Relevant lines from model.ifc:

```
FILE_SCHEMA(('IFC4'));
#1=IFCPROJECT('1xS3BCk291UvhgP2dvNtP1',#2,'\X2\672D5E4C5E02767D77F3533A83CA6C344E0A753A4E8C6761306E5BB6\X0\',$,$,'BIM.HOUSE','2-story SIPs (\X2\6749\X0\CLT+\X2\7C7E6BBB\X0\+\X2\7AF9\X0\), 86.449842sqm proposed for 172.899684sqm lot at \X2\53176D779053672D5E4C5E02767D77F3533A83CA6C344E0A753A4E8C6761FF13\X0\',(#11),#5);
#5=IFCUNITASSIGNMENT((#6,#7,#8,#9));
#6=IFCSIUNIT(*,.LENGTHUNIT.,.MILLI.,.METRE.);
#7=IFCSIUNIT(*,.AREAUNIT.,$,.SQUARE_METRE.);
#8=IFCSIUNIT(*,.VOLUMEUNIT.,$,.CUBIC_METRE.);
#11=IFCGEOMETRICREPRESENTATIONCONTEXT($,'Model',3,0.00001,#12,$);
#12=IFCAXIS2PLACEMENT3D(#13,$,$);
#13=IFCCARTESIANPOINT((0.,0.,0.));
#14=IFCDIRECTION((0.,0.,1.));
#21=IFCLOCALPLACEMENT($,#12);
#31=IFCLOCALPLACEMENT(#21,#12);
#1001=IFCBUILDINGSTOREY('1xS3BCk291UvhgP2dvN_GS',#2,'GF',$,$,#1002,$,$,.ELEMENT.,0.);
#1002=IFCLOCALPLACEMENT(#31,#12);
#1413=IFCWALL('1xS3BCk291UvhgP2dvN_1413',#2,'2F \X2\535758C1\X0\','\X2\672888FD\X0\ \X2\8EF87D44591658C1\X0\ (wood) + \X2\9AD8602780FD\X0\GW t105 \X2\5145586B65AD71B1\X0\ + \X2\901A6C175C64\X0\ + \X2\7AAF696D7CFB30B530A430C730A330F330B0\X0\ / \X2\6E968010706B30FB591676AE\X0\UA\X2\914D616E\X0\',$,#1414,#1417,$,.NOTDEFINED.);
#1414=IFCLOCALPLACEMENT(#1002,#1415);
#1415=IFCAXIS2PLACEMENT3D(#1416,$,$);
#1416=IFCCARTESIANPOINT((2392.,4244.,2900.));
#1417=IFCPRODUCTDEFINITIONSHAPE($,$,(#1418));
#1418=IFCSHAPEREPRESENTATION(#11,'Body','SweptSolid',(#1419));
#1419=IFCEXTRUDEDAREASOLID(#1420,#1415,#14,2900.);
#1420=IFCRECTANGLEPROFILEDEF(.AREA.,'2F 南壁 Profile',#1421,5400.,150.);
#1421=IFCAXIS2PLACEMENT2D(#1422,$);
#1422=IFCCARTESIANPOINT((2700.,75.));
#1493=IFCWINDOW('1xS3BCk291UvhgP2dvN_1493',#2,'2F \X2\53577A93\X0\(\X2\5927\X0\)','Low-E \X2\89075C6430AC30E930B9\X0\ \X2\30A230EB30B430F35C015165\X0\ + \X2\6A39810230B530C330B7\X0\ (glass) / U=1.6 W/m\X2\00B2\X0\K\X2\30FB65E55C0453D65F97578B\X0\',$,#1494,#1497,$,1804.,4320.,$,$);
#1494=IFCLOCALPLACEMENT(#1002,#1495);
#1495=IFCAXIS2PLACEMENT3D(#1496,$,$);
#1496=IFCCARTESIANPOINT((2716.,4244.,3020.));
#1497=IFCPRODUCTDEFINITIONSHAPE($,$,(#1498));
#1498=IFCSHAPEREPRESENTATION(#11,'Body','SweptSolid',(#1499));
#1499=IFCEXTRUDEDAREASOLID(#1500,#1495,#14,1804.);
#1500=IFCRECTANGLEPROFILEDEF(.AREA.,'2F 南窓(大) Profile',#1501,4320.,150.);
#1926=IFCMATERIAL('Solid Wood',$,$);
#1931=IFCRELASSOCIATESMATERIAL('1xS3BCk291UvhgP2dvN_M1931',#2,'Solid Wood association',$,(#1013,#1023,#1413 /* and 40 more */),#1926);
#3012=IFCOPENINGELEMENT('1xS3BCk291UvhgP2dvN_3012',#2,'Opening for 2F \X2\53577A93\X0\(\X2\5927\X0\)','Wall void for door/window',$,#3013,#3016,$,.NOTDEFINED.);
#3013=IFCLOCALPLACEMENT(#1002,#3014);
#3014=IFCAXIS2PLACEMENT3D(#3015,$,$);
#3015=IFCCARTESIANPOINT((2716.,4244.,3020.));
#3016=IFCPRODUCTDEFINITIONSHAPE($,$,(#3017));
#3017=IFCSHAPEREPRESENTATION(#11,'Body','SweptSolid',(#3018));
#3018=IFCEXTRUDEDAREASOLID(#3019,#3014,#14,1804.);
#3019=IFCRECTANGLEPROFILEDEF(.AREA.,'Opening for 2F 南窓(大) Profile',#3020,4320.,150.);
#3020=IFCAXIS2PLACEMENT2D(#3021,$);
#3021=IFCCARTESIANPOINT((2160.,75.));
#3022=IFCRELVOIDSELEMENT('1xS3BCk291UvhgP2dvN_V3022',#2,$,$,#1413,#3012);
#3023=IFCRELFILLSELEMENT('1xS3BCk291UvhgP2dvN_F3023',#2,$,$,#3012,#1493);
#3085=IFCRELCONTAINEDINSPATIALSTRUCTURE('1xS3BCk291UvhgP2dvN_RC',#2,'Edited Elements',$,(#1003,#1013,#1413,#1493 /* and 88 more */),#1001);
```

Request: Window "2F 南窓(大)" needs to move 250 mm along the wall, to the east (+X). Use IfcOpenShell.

```python
import ifcopenshell
import ifcopenshell.api.geometry
import ifcopenshell.util.placement

model = ifcopenshell.open("model.ifc")

window = model.by_guid("1xS3BCk291UvhgP2dvN_1493")
opening = window.FillsVoids[0].RelatingOpeningElement
wall = opening.VoidsElements[0].RelatingBuildingElement

wall_matrix = ifcopenshell.util.placement.get_local_placement(wall.ObjectPlacement)
shift = wall_matrix[:3, 0] * 250.0
before = ifcopenshell.util.placement.get_local_placement(window.ObjectPlacement)[:3, 3].copy()

# The window is not placed relative to its opening, so move both.
for product in (opening, window):
    matrix = ifcopenshell.util.placement.get_local_placement(product.ObjectPlacement)
    matrix[:3, 3] += shift
    ifcopenshell.api.geometry.edit_object_placement(model, product=product, matrix=matrix, is_si=False)

after = ifcopenshell.util.placement.get_local_placement(window.ObjectPlacement)[:3, 3]
print("window moved by", (after - before).round(3) + 0.0)

model.write("model_rev.ifc")
```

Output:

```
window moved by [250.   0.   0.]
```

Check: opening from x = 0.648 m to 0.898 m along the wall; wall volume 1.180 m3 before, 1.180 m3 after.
